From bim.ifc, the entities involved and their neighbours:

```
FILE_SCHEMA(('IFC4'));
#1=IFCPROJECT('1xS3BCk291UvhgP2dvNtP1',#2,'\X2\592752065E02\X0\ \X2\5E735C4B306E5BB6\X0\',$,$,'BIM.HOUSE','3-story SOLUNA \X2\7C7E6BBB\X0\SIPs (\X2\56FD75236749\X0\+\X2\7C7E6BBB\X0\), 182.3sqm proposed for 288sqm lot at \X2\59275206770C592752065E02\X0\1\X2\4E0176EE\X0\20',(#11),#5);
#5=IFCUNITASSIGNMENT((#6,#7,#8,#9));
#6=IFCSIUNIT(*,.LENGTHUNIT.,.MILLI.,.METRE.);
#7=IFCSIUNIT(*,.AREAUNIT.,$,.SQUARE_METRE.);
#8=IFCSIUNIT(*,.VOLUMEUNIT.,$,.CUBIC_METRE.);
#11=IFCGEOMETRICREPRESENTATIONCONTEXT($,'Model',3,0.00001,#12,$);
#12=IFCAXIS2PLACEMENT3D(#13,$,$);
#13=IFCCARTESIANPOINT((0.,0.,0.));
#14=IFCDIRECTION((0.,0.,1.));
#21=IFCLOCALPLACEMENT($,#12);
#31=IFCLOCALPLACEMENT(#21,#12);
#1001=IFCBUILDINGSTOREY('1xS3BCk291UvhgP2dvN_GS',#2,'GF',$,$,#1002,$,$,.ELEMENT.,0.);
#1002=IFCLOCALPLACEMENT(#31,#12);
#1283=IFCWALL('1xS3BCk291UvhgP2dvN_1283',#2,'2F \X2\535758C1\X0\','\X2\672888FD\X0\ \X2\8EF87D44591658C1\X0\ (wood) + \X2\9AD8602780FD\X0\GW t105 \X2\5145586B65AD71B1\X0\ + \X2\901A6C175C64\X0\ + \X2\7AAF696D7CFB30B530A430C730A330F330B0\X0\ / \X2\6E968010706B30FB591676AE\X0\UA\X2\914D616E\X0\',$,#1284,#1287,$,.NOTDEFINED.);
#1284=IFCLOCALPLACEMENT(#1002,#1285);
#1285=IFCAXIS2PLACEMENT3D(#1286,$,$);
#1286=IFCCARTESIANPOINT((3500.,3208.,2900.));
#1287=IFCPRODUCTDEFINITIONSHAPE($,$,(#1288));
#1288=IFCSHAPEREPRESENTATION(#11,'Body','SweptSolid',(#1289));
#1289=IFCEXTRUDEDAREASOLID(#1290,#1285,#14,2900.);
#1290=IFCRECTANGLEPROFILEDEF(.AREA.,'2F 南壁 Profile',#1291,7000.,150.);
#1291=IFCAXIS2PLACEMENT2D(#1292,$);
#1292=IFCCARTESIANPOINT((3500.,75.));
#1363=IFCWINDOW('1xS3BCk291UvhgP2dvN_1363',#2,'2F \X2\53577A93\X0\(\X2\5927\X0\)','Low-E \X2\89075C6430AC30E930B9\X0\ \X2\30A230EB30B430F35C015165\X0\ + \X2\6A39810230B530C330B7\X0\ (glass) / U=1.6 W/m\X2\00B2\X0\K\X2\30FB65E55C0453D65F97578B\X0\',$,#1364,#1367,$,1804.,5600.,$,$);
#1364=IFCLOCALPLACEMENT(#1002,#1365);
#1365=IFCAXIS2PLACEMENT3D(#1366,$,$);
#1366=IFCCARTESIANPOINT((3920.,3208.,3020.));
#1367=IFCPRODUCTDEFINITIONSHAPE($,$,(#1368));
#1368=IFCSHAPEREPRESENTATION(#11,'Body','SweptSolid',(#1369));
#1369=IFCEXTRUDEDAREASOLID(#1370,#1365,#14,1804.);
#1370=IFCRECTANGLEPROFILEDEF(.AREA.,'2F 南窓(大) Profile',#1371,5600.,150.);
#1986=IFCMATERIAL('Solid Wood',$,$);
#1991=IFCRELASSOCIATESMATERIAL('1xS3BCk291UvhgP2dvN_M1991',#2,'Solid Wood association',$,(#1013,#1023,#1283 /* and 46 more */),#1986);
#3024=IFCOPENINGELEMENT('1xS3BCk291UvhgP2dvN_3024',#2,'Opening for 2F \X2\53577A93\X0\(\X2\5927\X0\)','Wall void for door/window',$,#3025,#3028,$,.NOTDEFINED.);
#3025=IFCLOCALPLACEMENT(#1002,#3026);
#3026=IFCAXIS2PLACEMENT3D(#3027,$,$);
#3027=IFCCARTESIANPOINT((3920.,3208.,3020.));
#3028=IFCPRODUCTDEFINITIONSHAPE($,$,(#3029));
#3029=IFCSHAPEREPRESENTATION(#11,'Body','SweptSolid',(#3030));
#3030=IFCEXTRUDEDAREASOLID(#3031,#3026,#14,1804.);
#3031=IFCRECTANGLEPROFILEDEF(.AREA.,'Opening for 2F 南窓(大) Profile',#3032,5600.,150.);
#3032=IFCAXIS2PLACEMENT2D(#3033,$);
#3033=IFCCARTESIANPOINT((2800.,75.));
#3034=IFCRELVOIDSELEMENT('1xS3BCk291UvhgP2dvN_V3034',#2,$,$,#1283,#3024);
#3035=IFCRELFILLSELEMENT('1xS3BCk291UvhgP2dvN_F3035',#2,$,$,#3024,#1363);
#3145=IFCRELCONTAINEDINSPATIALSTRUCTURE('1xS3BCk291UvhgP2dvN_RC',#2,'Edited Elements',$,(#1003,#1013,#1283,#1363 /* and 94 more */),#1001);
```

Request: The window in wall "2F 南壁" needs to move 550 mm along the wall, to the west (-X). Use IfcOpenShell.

```python
import ifcopenshell
import ifcopenshell.api.geometry
import ifcopenshell.util.placement
import ifcopenshell.util.unit

model = ifcopenshell.open("bim.ifc")
unit_scale = ifcopenshell.util.unit.calculate_unit_scale(model)

window = model.by_id(1363)
opening = window.FillsVoids[0].RelatingOpeningElement
wall = opening.VoidsElements[0].RelatingBuildingElement

wall_matrix = ifcopenshell.util.placement.get_local_placement(wall.ObjectPlacement)
shift = wall_matrix[:3, 0] * -0.55 / unit_scale
before = ifcopenshell.util.placement.get_local_placement(window.ObjectPlacement)[:3, 3].copy()

# The window is not placed relative to its opening, so move both.
for product in (opening, window):
    matrix = ifcopenshell.util.placement.get_local_placement(product.ObjectPlacement)
    matrix[:3, 3] += shift
    ifcopenshell.api.geometry.edit_object_placement(model, product=product, matrix=matrix, is_si=False)

after = ifcopenshell.util.placement.get_local_placement(window.ObjectPlacement)[:3, 3]
print("window moved by", (after - before).round(3) + 0.0)

model.write("bim_updated.ifc")
```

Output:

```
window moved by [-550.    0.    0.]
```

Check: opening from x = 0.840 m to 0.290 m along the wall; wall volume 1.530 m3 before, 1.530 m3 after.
